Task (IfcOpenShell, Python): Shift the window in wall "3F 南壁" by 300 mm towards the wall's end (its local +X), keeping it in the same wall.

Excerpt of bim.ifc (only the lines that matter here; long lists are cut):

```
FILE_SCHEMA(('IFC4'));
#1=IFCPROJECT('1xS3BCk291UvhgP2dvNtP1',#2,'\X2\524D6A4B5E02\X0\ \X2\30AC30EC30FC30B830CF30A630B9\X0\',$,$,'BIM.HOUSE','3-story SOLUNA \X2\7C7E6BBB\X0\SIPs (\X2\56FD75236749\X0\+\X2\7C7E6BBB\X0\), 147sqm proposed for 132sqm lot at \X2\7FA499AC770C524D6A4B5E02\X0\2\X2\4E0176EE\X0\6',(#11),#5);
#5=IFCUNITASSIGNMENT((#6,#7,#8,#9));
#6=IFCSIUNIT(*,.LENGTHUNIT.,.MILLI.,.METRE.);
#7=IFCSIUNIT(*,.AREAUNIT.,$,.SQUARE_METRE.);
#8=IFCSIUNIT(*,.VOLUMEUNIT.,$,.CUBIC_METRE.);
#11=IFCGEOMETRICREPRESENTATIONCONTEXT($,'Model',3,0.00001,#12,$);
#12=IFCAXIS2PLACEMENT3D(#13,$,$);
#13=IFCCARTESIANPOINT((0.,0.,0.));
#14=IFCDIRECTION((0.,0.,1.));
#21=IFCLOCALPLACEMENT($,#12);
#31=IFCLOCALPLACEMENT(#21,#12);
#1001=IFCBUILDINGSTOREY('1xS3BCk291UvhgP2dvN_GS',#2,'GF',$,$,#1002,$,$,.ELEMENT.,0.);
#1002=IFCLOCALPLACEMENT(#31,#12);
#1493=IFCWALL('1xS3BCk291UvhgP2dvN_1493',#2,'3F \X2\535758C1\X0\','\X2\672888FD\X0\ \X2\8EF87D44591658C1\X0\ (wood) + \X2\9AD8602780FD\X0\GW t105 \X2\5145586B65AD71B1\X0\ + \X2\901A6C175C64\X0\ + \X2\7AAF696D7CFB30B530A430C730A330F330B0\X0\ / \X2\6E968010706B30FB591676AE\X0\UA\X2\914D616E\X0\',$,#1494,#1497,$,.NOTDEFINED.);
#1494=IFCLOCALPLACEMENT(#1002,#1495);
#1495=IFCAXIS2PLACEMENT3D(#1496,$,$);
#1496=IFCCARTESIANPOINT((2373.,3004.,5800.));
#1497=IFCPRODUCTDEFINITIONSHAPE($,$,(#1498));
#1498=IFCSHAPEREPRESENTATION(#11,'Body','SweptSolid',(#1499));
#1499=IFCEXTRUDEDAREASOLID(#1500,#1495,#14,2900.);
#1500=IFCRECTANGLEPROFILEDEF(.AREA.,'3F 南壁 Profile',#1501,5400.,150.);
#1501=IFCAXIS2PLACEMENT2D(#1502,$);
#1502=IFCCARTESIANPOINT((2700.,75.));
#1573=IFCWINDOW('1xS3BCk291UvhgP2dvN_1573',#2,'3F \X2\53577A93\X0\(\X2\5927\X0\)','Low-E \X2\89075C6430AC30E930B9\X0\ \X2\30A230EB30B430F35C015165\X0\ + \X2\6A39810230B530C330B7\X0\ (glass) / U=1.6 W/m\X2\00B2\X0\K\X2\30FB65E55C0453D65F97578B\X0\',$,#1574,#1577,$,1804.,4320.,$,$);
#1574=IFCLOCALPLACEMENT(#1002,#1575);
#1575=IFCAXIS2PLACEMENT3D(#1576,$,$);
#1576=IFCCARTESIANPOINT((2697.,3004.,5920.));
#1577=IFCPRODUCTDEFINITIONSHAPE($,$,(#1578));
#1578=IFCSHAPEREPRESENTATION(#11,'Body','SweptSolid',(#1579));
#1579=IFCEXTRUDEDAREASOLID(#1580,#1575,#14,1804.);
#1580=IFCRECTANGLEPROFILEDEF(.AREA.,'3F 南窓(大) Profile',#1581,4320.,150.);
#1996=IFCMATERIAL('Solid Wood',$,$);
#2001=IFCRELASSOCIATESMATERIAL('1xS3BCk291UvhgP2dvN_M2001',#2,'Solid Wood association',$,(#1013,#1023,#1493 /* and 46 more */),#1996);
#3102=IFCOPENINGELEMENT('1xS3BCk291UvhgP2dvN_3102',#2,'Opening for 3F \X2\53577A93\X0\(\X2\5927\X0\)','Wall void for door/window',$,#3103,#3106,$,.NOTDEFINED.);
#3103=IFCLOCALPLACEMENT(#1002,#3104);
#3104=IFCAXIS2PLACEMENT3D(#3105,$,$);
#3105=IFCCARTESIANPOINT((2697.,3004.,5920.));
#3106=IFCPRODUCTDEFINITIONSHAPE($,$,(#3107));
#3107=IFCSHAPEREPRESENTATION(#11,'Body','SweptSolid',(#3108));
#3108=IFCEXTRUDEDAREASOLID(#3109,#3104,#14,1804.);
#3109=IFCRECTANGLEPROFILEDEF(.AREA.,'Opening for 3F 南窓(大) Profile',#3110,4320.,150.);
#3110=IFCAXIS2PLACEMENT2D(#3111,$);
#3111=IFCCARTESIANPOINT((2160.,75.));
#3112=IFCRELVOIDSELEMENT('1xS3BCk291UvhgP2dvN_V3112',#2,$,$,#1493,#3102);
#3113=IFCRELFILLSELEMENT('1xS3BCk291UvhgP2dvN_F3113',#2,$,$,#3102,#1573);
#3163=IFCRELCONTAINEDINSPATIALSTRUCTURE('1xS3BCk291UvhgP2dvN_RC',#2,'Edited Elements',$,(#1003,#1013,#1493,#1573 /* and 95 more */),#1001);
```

```python
import ifcopenshell
import ifcopenshell.api.geometry
import ifcopenshell.util.placement

model = ifcopenshell.open("bim.ifc")

window = model.by_guid("1xS3BCk291UvhgP2dvN_1573")
opening = window.FillsVoids[0].RelatingOpeningElement
wall = opening.VoidsElements[0].RelatingBuildingElement

wall_matrix = ifcopenshell.util.placement.get_local_placement(wall.ObjectPlacement)
shift = wall_matrix[:3, 0] * 300.0
before = ifcopenshell.util.placement.get_local_placement(window.ObjectPlacement)[:3, 3].copy()

# The window is not placed relative to its opening, so move both.
for product in (opening, window):
    matrix = ifcopenshell.util.placement.get_local_placement(product.ObjectPlacement)
    matrix[:3, 3] += shift
    ifcopenshell.api.geometry.edit_object_placement(model, product=product, matrix=matrix, is_si=False)

after = ifcopenshell.util.placement.get_local_placement(window.ObjectPlacement)[:3, 3]
print("window moved by", (after - before).round(3) + 0.0)

model.write("bim_updated.ifc")
```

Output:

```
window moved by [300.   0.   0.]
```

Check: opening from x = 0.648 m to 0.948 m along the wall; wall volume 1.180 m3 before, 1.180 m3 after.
